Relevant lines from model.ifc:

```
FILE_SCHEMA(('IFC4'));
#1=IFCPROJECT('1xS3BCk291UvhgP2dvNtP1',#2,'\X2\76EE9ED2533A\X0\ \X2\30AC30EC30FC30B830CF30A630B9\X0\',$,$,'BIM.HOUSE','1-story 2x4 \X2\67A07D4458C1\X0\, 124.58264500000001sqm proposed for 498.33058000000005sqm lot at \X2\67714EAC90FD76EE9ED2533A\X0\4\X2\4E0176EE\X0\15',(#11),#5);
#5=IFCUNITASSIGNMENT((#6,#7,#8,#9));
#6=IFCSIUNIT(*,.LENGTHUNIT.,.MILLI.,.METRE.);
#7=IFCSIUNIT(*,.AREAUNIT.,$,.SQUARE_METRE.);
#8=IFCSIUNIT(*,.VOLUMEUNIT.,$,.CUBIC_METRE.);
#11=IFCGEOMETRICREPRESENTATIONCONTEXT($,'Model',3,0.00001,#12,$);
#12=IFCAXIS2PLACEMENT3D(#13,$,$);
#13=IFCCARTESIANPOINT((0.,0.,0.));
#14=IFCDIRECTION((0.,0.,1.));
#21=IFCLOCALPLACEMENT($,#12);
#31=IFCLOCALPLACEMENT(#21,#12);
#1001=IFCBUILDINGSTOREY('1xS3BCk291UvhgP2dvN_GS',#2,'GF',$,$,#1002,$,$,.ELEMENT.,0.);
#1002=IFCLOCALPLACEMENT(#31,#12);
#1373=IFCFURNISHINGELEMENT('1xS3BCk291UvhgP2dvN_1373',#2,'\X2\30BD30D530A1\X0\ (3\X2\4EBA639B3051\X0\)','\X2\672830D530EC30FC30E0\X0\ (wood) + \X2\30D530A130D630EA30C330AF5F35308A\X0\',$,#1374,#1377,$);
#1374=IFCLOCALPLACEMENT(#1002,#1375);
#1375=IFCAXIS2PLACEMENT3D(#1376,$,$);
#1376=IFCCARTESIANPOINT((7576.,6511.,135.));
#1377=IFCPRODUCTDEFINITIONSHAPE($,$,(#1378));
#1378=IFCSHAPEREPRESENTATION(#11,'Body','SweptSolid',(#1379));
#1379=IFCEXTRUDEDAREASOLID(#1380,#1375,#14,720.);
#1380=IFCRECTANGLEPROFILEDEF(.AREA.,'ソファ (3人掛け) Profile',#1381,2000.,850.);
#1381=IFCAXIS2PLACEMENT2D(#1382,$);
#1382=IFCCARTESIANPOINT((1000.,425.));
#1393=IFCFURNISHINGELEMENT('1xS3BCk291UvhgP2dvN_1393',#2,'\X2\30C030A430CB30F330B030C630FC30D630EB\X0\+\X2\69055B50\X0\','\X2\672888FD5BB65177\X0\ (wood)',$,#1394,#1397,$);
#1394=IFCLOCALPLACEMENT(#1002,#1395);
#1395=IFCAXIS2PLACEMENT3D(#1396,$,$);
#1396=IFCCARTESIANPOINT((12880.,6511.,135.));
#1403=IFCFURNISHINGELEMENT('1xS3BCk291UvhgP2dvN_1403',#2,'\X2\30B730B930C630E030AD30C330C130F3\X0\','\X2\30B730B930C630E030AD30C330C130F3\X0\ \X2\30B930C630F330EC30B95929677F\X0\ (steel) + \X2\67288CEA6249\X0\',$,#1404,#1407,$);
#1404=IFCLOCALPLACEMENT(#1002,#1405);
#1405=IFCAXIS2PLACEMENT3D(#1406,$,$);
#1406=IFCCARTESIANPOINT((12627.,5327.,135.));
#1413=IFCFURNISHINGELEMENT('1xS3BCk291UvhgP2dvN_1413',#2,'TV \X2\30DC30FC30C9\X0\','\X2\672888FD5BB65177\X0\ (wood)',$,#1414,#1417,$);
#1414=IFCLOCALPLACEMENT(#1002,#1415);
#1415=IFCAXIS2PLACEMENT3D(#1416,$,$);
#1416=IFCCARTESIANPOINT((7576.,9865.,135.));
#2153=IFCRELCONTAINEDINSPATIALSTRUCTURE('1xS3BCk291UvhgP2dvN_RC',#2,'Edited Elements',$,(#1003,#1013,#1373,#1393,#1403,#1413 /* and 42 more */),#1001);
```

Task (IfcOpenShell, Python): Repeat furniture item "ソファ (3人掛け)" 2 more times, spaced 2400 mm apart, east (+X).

```python
import numpy as np
import ifcopenshell
import ifcopenshell.api.geometry
import ifcopenshell.api.root
import ifcopenshell.util.element
import ifcopenshell.util.placement

model = ifcopenshell.open("model.ifc")


def reuse_history(source, copy):
    """copy_class also copies each property set's owner history, people and application; keep the originals."""
    for rel in copy.IsDefinedBy:
        if rel.is_a("IfcRelDefinesByProperties") and (history := rel.RelatingPropertyDefinition.OwnerHistory):
            rel.RelatingPropertyDefinition.OwnerHistory = source.OwnerHistory
            ifcopenshell.util.element.remove_deep2(model, history)


source = model.by_id(1373)
base = ifcopenshell.util.placement.get_local_placement(source.ObjectPlacement)
step = np.array([1.0, 0.0, 0.0]) * 2400.0

for i in range(1, 3):
    copy = ifcopenshell.api.root.copy_class(model, product=source)
    copy.Representation = ifcopenshell.util.element.copy_deep(
        model, source.Representation, exclude=["IfcGeometricRepresentationContext", "IfcRepresentationMap"]
    )
    reuse_history(source, copy)
    matrix = base.copy()
    matrix[:3, 3] += i * step
    print("added at", matrix[:3, 3].round(3) + 0.0)
    ifcopenshell.api.geometry.edit_object_placement(model, product=copy, matrix=matrix, is_si=False)

model.write("model_v2.ifc")
```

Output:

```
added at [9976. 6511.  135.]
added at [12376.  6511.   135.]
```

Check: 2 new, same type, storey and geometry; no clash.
